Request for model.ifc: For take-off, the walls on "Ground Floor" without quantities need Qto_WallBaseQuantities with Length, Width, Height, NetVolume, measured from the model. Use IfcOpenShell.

First a look at what the model holds.

```python
import ifcopenshell
import ifcopenshell.util.element
import ifcopenshell.util.unit

model = ifcopenshell.open("model.ifc")
print(model.schema)
for unit_type in ("LENGTHUNIT", "AREAUNIT", "VOLUMEUNIT"):
    print(unit_type, ifcopenshell.util.unit.calculate_unit_scale(model, unit_type))
storey = next(s for s in model.by_type("IfcBuildingStorey") if s.Name == "Ground Floor")
walls = [e for e in ifcopenshell.util.element.get_decomposition(storey) if e.is_a("IfcWall")]
for e in sorted(walls, key=lambda e: e.id()):
    print(e.id(), e.is_a(), e.Name, list(ifcopenshell.util.element.get_psets(e, qtos_only=True)), sep=" | ")
```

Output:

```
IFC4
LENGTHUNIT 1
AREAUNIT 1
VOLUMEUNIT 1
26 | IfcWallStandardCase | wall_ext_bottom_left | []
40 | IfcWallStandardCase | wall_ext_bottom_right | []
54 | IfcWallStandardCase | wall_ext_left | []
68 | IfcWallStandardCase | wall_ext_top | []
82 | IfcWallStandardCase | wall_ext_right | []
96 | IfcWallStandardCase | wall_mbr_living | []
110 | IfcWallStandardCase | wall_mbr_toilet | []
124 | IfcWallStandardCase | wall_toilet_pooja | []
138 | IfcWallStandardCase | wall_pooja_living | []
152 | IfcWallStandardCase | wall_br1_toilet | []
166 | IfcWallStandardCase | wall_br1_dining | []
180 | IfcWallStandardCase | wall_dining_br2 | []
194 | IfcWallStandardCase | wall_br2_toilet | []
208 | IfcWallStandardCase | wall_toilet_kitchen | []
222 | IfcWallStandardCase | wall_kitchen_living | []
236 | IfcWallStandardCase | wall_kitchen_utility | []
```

```python
import ifcopenshell
import ifcopenshell.api.pset
import ifcopenshell.geom
import ifcopenshell.util.element
import ifcopenshell.util.shape
import ifcopenshell.util.unit

model = ifcopenshell.open("model.ifc")
unit_scale = ifcopenshell.util.unit.calculate_unit_scale(model)
volume_scale = ifcopenshell.util.unit.calculate_unit_scale(model, "VOLUMEUNIT")
settings = ifcopenshell.geom.settings()

storey = next(s for s in model.by_type("IfcBuildingStorey") if s.Name == "Ground Floor")
walls = [e for e in ifcopenshell.util.element.get_decomposition(storey) if e.is_a("IfcWall")]

for e in sorted(walls, key=lambda e: e.id()):
    if ifcopenshell.util.element.get_psets(e, qtos_only=True, should_inherit=False):
        continue
    # Geometry comes back in metres, in the element's own axes.
    shape = ifcopenshell.geom.create_shape(settings, e)
    values = {
        "Length": ifcopenshell.util.shape.get_x(shape.geometry) / unit_scale,
        "Width": ifcopenshell.util.shape.get_y(shape.geometry) / unit_scale,
        "Height": ifcopenshell.util.shape.get_z(shape.geometry) / unit_scale,
        "NetVolume": ifcopenshell.util.shape.get_volume(shape.geometry) / volume_scale,
    }
    qto = ifcopenshell.api.pset.add_qto(model, product=e, name="Qto_WallBaseQuantities")
    ifcopenshell.api.pset.edit_qto(model, qto=qto, properties=values)
    print(e.id(), {k: round(v, 3) for k, v in values.items()})

model.write("model_v2.ifc")
```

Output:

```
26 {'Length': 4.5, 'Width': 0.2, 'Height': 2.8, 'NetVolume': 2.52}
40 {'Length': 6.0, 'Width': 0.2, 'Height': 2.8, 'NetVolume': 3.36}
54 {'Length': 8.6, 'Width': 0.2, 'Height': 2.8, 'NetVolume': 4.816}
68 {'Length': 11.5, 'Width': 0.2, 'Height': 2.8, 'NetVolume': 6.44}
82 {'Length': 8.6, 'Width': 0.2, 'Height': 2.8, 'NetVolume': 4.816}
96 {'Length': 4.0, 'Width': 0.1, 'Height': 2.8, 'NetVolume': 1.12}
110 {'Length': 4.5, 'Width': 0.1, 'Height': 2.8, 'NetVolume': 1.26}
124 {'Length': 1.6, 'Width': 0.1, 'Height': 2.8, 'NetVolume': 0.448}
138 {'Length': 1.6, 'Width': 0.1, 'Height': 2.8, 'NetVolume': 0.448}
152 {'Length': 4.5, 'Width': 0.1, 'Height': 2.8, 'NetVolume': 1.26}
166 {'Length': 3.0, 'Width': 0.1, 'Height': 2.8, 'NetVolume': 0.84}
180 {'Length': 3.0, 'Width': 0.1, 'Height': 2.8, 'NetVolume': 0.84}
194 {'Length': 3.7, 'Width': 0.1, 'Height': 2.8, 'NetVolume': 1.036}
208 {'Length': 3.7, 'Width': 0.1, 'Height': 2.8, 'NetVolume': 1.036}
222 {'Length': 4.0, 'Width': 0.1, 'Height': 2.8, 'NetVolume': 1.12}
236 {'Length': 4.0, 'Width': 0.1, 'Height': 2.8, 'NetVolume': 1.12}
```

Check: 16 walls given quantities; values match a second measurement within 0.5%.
